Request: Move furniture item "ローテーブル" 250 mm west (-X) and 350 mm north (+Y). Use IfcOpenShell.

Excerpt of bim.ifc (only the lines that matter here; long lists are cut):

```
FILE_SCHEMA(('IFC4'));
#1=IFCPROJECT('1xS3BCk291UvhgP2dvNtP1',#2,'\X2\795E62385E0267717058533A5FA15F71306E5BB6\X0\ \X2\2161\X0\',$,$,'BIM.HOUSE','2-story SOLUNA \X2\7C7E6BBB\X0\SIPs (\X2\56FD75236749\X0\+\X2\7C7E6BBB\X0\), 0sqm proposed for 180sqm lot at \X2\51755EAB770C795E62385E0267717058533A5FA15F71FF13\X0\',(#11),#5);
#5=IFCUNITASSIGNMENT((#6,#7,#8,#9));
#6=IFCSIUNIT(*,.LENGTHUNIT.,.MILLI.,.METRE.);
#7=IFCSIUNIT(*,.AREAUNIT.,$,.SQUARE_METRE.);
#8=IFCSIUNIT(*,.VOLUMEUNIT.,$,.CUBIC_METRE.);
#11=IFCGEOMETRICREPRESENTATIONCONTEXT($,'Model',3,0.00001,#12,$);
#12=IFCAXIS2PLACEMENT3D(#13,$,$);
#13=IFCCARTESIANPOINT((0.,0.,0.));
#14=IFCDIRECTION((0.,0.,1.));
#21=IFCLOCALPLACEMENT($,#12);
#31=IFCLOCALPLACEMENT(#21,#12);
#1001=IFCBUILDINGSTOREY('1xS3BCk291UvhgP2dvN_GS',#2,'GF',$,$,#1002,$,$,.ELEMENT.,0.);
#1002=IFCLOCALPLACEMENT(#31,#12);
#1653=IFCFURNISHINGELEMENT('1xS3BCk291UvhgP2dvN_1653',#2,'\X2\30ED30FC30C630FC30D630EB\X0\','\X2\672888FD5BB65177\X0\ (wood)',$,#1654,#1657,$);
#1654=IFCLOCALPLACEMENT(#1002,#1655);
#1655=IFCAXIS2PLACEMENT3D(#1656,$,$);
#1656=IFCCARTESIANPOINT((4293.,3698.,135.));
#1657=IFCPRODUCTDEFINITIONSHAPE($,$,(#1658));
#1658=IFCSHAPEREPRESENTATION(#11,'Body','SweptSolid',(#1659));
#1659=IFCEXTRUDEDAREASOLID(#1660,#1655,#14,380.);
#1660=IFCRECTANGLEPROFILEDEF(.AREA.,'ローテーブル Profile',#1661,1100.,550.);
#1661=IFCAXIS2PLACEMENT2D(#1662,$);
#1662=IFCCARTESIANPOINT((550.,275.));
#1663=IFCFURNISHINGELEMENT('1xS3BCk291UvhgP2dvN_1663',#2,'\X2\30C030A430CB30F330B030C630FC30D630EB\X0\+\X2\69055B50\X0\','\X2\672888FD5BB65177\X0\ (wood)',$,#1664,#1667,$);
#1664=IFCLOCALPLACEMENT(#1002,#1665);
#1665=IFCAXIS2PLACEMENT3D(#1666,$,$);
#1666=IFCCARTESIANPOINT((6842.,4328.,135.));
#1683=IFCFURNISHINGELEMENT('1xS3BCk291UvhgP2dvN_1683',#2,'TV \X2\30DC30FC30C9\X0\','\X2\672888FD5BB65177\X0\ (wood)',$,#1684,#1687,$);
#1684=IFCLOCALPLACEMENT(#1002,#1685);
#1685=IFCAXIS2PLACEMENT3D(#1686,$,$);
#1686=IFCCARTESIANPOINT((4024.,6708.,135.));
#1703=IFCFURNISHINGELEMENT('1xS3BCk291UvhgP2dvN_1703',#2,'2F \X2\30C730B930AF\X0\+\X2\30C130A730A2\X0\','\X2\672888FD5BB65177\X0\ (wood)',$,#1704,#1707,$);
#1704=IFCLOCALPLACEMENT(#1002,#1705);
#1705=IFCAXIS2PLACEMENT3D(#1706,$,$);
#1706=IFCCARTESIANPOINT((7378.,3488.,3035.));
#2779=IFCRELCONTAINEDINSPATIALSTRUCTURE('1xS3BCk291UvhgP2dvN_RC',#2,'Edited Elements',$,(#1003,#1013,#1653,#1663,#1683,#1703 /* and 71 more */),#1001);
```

```python
import ifcopenshell
import ifcopenshell.api.geometry
import ifcopenshell.util.placement
import ifcopenshell.util.unit

model = ifcopenshell.open("bim.ifc")
unit_scale = ifcopenshell.util.unit.calculate_unit_scale(model)

item = model.by_id(1653)
matrix = ifcopenshell.util.placement.get_local_placement(item.ObjectPlacement)
matrix[0, 3] -= 0.25 / unit_scale
matrix[1, 3] += 0.35 / unit_scale
ifcopenshell.api.geometry.edit_object_placement(model, product=item, matrix=matrix, is_si=False)

print(ifcopenshell.util.placement.get_local_placement(item.ObjectPlacement).round(3) + 0.0)

model.write("bim_v2.ifc")
```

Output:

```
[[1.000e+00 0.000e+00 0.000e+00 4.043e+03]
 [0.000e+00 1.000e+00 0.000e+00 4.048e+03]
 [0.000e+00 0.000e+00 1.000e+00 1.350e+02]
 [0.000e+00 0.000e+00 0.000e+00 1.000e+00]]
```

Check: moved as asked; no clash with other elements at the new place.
